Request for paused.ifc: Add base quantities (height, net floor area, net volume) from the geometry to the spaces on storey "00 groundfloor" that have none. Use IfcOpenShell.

First a look at what the model holds.

```python
import ifcopenshell
import ifcopenshell.util.element
import ifcopenshell.util.unit

model = ifcopenshell.open("paused.ifc")
print(model.schema)
for unit_type in ("LENGTHUNIT", "AREAUNIT", "VOLUMEUNIT"):
    print(unit_type, ifcopenshell.util.unit.calculate_unit_scale(model, unit_type))
storey = next(s for s in model.by_type("IfcBuildingStorey") if s.Name == "00 groundfloor")
spaces = [e for e in ifcopenshell.util.element.get_decomposition(storey) if e.is_a("IfcSpace")]
for e in sorted(spaces, key=lambda e: e.id()):
    print(e.id(), e.is_a(), e.Name, list(ifcopenshell.util.element.get_psets(e, qtos_only=True)), sep=" | ")
```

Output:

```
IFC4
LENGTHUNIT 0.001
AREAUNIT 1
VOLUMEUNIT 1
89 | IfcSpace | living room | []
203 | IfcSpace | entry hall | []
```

```python
import ifcopenshell
import ifcopenshell.api.pset
import ifcopenshell.geom
import ifcopenshell.util.element
import ifcopenshell.util.shape
import ifcopenshell.util.unit

model = ifcopenshell.open("paused.ifc")
unit_scale = ifcopenshell.util.unit.calculate_unit_scale(model)
area_scale = ifcopenshell.util.unit.calculate_unit_scale(model, "AREAUNIT")
volume_scale = ifcopenshell.util.unit.calculate_unit_scale(model, "VOLUMEUNIT")
settings = ifcopenshell.geom.settings()

storey = next(s for s in model.by_type("IfcBuildingStorey") if s.Name == "00 groundfloor")
spaces = [e for e in ifcopenshell.util.element.get_decomposition(storey) if e.is_a("IfcSpace")]

for e in sorted(spaces, key=lambda e: e.id()):
    if ifcopenshell.util.element.get_psets(e, qtos_only=True, should_inherit=False):
        continue
    # Geometry comes back in metres, in the element's own axes.
    shape = ifcopenshell.geom.create_shape(settings, e)
    values = {
        "Height": ifcopenshell.util.shape.get_z(shape.geometry) / unit_scale,
        "NetFloorArea": ifcopenshell.util.shape.get_footprint_area(shape.geometry) / area_scale,
        "NetVolume": ifcopenshell.util.shape.get_volume(shape.geometry) / volume_scale,
    }
    qto = ifcopenshell.api.pset.add_qto(model, product=e, name="Qto_SpaceBaseQuantities")
    ifcopenshell.api.pset.edit_qto(model, qto=qto, properties=values)
    print(e.id(), {k: round(v, 3) for k, v in values.items()})

model.write("paused_v2.ifc")
```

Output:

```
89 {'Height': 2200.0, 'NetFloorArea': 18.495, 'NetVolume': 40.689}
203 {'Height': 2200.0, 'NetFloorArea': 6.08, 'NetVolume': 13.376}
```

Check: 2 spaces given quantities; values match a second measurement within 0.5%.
